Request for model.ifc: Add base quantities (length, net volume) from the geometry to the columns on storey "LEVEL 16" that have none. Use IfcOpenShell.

First a look at what the model holds.

```python
import ifcopenshell
import ifcopenshell.util.element
import ifcopenshell.util.unit

model = ifcopenshell.open("model.ifc")
print(model.schema)
for unit_type in ("LENGTHUNIT", "AREAUNIT", "VOLUMEUNIT"):
    print(unit_type, ifcopenshell.util.unit.calculate_unit_scale(model, unit_type))
storey = next(s for s in model.by_type("IfcBuildingStorey") if s.Name == "LEVEL 16")
columns = [e for e in ifcopenshell.util.element.get_decomposition(storey) if e.is_a("IfcColumn")]
for e in sorted(columns, key=lambda e: e.id()):
    print(e.id(), e.is_a(), e.Name, list(ifcopenshell.util.element.get_psets(e, qtos_only=True)), sep=" | ")
```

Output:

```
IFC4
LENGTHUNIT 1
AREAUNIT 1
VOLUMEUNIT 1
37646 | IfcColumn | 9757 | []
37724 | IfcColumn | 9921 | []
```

```python
import ifcopenshell
import ifcopenshell.api.pset
import ifcopenshell.geom
import ifcopenshell.util.element
import ifcopenshell.util.shape
import ifcopenshell.util.unit

model = ifcopenshell.open("model.ifc")
unit_scale = ifcopenshell.util.unit.calculate_unit_scale(model)
volume_scale = ifcopenshell.util.unit.calculate_unit_scale(model, "VOLUMEUNIT")
settings = ifcopenshell.geom.settings()

storey = next(s for s in model.by_type("IfcBuildingStorey") if s.Name == "LEVEL 16")
columns = [e for e in ifcopenshell.util.element.get_decomposition(storey) if e.is_a("IfcColumn")]

for e in sorted(columns, key=lambda e: e.id()):
    if ifcopenshell.util.element.get_psets(e, qtos_only=True, should_inherit=False):
        continue
    # Geometry comes back in metres, in the element's own axes.
    shape = ifcopenshell.geom.create_shape(settings, e)
    values = {
        "Length": ifcopenshell.util.shape.get_z(shape.geometry) / unit_scale,
        "NetVolume": ifcopenshell.util.shape.get_volume(shape.geometry) / volume_scale,
    }
    qto = ifcopenshell.api.pset.add_qto(model, product=e, name="Qto_ColumnBaseQuantities")
    ifcopenshell.api.pset.edit_qto(model, qto=qto, properties=values)
    print(e.id(), {k: round(v, 3) for k, v in values.items()})

model.write("model-out.ifc")
```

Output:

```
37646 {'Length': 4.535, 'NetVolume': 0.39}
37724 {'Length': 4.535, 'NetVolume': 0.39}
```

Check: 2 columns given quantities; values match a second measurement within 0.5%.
